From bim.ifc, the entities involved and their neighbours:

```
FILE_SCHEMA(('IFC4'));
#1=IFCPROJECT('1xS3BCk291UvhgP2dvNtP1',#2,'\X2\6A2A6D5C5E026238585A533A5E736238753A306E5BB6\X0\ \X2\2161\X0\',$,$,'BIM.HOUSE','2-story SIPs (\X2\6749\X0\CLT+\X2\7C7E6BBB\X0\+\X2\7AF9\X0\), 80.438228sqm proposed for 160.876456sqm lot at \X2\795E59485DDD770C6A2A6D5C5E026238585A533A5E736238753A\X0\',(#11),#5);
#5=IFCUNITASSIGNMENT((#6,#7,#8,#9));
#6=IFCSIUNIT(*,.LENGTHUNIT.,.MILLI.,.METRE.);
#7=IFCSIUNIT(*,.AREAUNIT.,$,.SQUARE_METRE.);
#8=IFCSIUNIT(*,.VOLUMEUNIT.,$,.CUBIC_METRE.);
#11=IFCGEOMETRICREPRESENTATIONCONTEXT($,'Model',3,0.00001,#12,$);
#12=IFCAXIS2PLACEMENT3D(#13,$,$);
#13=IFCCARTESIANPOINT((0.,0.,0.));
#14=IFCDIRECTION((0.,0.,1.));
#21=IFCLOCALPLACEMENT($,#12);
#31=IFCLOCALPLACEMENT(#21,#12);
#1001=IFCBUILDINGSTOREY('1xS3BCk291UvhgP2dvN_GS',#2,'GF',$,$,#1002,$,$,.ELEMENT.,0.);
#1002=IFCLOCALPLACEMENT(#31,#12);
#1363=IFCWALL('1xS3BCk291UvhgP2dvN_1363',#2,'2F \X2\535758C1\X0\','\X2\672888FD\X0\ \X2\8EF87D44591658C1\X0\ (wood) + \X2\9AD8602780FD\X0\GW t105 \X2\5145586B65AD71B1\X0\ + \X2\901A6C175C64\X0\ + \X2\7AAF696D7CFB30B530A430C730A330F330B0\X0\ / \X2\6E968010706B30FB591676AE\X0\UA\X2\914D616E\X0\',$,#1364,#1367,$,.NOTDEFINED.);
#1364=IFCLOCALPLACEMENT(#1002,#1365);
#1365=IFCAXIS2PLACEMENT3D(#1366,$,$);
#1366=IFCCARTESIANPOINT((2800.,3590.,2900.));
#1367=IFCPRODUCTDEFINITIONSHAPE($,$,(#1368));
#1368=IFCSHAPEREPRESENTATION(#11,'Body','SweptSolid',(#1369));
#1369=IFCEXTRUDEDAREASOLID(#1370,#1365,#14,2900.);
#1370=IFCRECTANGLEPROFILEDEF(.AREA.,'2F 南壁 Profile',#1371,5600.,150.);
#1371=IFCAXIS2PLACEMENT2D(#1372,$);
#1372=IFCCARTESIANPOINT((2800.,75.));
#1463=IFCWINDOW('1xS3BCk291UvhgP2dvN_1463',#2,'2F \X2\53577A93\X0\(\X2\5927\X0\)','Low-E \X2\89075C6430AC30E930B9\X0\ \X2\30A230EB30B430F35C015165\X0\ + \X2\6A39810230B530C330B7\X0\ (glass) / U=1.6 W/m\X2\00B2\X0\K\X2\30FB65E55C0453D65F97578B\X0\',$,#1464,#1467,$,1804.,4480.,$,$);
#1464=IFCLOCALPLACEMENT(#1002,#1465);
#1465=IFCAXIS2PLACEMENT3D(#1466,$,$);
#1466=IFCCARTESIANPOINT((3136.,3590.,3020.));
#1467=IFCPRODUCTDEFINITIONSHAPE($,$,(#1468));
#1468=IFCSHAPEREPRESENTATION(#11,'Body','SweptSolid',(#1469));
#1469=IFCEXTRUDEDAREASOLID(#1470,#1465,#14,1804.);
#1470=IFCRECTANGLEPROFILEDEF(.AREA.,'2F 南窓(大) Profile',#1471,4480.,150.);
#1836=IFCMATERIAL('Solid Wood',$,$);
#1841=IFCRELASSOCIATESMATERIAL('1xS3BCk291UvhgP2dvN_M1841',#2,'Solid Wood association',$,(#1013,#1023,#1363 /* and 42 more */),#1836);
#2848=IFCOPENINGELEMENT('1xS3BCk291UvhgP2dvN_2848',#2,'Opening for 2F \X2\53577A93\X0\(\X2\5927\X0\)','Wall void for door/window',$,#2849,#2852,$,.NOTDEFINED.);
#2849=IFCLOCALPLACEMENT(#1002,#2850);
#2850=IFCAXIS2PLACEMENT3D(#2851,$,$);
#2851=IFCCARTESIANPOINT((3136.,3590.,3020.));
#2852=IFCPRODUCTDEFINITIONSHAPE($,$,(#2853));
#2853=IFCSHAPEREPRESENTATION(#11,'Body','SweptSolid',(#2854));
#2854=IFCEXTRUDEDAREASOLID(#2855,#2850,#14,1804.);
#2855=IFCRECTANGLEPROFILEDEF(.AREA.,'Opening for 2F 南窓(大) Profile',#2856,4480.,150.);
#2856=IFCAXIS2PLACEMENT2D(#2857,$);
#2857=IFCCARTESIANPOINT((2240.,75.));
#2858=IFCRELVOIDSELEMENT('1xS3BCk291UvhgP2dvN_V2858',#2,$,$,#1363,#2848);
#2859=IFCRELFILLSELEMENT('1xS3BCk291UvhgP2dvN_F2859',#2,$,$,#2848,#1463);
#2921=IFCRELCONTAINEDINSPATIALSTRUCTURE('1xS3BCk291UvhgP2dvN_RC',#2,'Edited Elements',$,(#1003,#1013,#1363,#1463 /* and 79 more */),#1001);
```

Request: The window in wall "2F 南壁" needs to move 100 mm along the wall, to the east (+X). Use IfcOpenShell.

```python
import ifcopenshell
import ifcopenshell.api.geometry
import ifcopenshell.util.placement

model = ifcopenshell.open("bim.ifc")

window = model.by_guid("1xS3BCk291UvhgP2dvN_1463")
opening = window.FillsVoids[0].RelatingOpeningElement
wall = opening.VoidsElements[0].RelatingBuildingElement

wall_matrix = ifcopenshell.util.placement.get_local_placement(wall.ObjectPlacement)
shift = wall_matrix[:3, 0] * 100.0
before = ifcopenshell.util.placement.get_local_placement(window.ObjectPlacement)[:3, 3].copy()

# The window is not placed relative to its opening, so move both.
for product in (opening, window):
    matrix = ifcopenshell.util.placement.get_local_placement(product.ObjectPlacement)
    matrix[:3, 3] += shift
    ifcopenshell.api.geometry.edit_object_placement(model, product=product, matrix=matrix, is_si=False)

after = ifcopenshell.util.placement.get_local_placement(window.ObjectPlacement)[:3, 3]
print("window moved by", (after - before).round(3) + 0.0)

model.write("bim_edited.ifc")
```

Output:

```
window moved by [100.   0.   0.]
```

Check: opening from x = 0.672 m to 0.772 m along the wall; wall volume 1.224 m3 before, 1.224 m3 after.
